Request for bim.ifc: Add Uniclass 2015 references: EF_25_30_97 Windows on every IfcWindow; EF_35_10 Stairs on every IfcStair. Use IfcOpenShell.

First a look at what the model holds.

```python
import ifcopenshell

model = ifcopenshell.open("bim.ifc")
print(model.schema)
print("classifications:", [c.Name for c in model.by_type("IfcClassification")])
for ifc_class in ("IfcDoor", "IfcRoof", "IfcStair", "IfcWall", "IfcWindow"):
    print(ifc_class, len(model.by_type(ifc_class)))
```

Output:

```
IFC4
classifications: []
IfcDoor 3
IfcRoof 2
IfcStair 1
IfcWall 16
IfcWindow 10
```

```python
import ifcopenshell
import ifcopenshell.api.classification

model = ifcopenshell.open("bim.ifc")

system = ifcopenshell.api.classification.add_classification(model, classification="Uniclass 2015")

codes = {
    "IfcWindow": ("EF_25_30_97", "Windows"),
    "IfcStair": ("EF_35_10", "Stairs"),
}
for ifc_class, (code, name) in codes.items():
    products = model.by_type(ifc_class)
    ifcopenshell.api.classification.add_reference(
        model, products=products, classification=system, identification=code, name=name
    )
    print(code, len(products))

model.write("bim_v2.ifc")
```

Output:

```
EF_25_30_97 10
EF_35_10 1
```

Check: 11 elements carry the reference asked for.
